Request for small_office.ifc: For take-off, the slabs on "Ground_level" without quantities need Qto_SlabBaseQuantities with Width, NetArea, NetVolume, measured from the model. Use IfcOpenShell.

First a look at what the model holds.

```python
import ifcopenshell
import ifcopenshell.util.element
import ifcopenshell.util.unit

model = ifcopenshell.open("small_office.ifc")
print(model.schema)
for unit_type in ("LENGTHUNIT", "AREAUNIT", "VOLUMEUNIT"):
    print(unit_type, ifcopenshell.util.unit.calculate_unit_scale(model, unit_type))
storey = next(s for s in model.by_type("IfcBuildingStorey") if s.Name == "Ground_level")
slabs = [e for e in ifcopenshell.util.element.get_decomposition(storey) if e.is_a("IfcSlab")]
for e in sorted(slabs, key=lambda e: e.id()):
    print(e.id(), e.is_a(), e.Name, list(ifcopenshell.util.element.get_psets(e, qtos_only=True)), sep=" | ")
```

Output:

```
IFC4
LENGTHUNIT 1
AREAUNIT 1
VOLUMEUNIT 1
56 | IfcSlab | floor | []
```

```python
import ifcopenshell
import ifcopenshell.api.pset
import ifcopenshell.geom
import ifcopenshell.util.element
import ifcopenshell.util.shape
import ifcopenshell.util.unit

model = ifcopenshell.open("small_office.ifc")
unit_scale = ifcopenshell.util.unit.calculate_unit_scale(model)
area_scale = ifcopenshell.util.unit.calculate_unit_scale(model, "AREAUNIT")
volume_scale = ifcopenshell.util.unit.calculate_unit_scale(model, "VOLUMEUNIT")
settings = ifcopenshell.geom.settings()

storey = next(s for s in model.by_type("IfcBuildingStorey") if s.Name == "Ground_level")
slabs = [e for e in ifcopenshell.util.element.get_decomposition(storey) if e.is_a("IfcSlab")]

for e in sorted(slabs, key=lambda e: e.id()):
    if ifcopenshell.util.element.get_psets(e, qtos_only=True, should_inherit=False):
        continue
    # Geometry comes back in metres, in the element's own axes.
    shape = ifcopenshell.geom.create_shape(settings, e)
    values = {
        "Width": ifcopenshell.util.shape.get_z(shape.geometry) / unit_scale,
        "NetArea": ifcopenshell.util.shape.get_footprint_area(shape.geometry) / area_scale,
        "NetVolume": ifcopenshell.util.shape.get_volume(shape.geometry) / volume_scale,
    }
    qto = ifcopenshell.api.pset.add_qto(model, product=e, name="Qto_SlabBaseQuantities")
    ifcopenshell.api.pset.edit_qto(model, qto=qto, properties=values)
    print(e.id(), {k: round(v, 3) for k, v in values.items()})

model.write("small_office-out.ifc")
```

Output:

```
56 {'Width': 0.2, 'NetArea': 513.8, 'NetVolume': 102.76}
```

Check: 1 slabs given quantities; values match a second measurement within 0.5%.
